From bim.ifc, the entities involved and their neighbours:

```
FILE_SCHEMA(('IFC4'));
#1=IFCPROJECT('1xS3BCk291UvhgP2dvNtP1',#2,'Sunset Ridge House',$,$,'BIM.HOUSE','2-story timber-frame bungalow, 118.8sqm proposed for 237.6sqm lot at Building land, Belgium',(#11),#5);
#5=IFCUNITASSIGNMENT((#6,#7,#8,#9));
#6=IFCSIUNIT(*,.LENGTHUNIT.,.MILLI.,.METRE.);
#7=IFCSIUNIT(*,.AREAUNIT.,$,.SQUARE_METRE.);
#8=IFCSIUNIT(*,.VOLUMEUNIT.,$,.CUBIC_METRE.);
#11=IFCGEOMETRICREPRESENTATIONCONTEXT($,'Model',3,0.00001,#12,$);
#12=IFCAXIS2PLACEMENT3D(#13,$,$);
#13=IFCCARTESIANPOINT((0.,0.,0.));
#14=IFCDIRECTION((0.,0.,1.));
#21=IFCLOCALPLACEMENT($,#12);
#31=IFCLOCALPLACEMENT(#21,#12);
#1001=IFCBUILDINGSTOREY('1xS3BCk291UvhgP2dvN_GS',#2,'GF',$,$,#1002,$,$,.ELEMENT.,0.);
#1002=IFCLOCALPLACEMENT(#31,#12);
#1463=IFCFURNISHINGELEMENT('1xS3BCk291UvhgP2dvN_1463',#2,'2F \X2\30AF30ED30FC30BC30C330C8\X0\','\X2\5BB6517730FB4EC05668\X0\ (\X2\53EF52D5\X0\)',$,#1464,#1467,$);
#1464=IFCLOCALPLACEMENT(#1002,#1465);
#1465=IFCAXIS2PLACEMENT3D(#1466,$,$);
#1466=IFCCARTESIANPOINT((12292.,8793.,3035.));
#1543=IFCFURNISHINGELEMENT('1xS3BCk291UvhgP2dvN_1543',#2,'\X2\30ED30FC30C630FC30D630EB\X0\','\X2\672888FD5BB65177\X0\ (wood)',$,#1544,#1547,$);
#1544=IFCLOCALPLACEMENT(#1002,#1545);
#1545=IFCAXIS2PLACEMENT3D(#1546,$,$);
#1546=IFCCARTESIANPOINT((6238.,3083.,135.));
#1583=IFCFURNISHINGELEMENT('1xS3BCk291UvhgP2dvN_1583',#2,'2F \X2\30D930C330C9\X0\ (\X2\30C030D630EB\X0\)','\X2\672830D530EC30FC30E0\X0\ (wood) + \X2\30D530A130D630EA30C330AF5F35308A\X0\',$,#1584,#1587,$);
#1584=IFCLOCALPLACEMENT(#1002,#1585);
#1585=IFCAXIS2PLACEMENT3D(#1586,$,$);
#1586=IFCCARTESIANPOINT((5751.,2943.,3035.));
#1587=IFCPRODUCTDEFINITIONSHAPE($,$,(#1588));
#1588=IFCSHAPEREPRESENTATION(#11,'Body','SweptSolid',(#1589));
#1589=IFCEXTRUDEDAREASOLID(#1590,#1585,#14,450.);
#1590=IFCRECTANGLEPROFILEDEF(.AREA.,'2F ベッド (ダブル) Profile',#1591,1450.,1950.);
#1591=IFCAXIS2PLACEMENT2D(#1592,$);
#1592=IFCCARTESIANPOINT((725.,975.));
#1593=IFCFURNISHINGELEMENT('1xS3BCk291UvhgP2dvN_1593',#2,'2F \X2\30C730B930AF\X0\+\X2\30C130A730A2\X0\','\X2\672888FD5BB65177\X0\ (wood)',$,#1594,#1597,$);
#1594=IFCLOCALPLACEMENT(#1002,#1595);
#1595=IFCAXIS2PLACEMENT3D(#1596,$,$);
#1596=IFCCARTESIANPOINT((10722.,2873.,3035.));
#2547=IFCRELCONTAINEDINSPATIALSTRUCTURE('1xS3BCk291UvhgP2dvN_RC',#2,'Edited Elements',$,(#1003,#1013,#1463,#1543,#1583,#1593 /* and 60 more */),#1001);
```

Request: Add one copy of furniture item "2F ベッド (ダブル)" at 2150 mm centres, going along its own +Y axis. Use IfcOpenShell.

```python
import ifcopenshell
import ifcopenshell.api.geometry
import ifcopenshell.api.root
import ifcopenshell.util.element
import ifcopenshell.util.placement

model = ifcopenshell.open("bim.ifc")


def reuse_history(source, copy):
    """copy_class also copies each property set's owner history, people and application; keep the originals."""
    for rel in copy.IsDefinedBy:
        if rel.is_a("IfcRelDefinesByProperties") and (history := rel.RelatingPropertyDefinition.OwnerHistory):
            rel.RelatingPropertyDefinition.OwnerHistory = source.OwnerHistory
            ifcopenshell.util.element.remove_deep2(model, history)


source = model.by_guid("1xS3BCk291UvhgP2dvN_1583")
base = ifcopenshell.util.placement.get_local_placement(source.ObjectPlacement)
step = base[:3, 1] * 2150.0

for i in range(1, 2):
    copy = ifcopenshell.api.root.copy_class(model, product=source)
    copy.Representation = ifcopenshell.util.element.copy_deep(
        model, source.Representation, exclude=["IfcGeometricRepresentationContext", "IfcRepresentationMap"]
    )
    reuse_history(source, copy)
    matrix = base.copy()
    matrix[:3, 3] += i * step
    print("added at", matrix[:3, 3].round(3) + 0.0)
    ifcopenshell.api.geometry.edit_object_placement(model, product=copy, matrix=matrix, is_si=False)

model.write("bim-out.ifc")
```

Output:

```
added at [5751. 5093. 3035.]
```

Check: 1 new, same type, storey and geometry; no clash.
